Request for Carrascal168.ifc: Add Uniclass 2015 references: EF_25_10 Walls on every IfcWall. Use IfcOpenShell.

First a look at what the model holds.

```python
import ifcopenshell

model = ifcopenshell.open("Carrascal168.ifc")
print(model.schema)
print("classifications:", [c.Name for c in model.by_type("IfcClassification")])
for ifc_class in ("IfcDoor", "IfcRoof", "IfcStair", "IfcWall", "IfcWindow"):
    print(ifc_class, len(model.by_type(ifc_class)))
```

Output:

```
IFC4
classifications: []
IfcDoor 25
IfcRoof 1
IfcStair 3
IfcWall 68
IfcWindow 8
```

```python
import ifcopenshell
import ifcopenshell.api.classification

model = ifcopenshell.open("Carrascal168.ifc")

system = ifcopenshell.api.classification.add_classification(model, classification="Uniclass 2015")

codes = {
    "IfcWall": ("EF_25_10", "Walls"),
}
for ifc_class, (code, name) in codes.items():
    products = model.by_type(ifc_class)
    ifcopenshell.api.classification.add_reference(
        model, products=products, classification=system, identification=code, name=name
    )
    print(code, len(products))

model.write("Carrascal168_v2.ifc")
```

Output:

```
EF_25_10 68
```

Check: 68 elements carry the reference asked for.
